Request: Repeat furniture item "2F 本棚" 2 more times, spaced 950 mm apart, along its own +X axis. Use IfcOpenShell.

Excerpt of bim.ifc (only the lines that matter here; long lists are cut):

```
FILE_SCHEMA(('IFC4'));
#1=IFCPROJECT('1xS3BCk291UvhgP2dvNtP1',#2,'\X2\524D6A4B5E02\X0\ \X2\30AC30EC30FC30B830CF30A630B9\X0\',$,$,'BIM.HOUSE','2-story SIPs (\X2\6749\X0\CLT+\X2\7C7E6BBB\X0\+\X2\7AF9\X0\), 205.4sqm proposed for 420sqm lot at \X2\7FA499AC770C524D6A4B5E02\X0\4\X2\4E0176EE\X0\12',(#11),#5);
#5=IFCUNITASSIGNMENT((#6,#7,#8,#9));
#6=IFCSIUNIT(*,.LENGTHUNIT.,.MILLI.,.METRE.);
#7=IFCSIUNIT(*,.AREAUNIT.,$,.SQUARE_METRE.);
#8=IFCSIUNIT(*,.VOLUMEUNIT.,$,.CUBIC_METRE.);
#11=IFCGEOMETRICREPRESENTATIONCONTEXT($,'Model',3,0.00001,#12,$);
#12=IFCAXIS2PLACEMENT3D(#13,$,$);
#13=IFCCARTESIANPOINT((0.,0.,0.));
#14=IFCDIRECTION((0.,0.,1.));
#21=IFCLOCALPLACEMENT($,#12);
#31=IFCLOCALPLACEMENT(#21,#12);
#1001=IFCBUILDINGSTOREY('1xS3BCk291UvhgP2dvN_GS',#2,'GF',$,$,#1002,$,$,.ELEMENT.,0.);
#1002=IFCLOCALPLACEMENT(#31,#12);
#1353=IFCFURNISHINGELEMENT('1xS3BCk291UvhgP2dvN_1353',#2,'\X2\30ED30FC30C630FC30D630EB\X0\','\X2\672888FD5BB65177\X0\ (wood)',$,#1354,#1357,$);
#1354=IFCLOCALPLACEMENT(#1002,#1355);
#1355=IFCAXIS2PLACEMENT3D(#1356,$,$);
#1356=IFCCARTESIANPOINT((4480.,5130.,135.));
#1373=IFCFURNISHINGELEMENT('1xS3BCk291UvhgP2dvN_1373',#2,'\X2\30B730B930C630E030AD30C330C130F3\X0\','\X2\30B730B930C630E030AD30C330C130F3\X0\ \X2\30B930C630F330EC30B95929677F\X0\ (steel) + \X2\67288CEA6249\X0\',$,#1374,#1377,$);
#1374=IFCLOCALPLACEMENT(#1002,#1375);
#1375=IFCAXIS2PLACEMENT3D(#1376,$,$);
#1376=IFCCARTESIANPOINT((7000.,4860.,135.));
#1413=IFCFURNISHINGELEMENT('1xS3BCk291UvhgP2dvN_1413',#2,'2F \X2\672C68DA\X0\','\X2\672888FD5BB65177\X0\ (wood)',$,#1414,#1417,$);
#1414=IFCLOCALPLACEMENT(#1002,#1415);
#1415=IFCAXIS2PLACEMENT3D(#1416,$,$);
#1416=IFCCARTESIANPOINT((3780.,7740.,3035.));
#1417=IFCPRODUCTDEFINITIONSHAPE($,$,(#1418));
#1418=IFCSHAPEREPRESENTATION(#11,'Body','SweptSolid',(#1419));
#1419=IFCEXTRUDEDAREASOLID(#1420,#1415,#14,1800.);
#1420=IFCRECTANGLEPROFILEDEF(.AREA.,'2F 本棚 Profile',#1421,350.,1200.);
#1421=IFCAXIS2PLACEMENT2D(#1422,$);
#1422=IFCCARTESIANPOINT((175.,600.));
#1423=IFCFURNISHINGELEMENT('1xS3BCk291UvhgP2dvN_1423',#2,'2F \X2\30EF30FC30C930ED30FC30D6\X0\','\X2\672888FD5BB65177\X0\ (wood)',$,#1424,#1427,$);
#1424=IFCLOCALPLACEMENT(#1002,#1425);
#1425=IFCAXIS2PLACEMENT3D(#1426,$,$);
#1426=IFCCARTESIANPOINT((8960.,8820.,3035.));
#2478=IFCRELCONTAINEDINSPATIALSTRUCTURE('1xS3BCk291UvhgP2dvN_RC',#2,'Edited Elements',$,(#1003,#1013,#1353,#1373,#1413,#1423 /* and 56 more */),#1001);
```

```python
import ifcopenshell
import ifcopenshell.api.geometry
import ifcopenshell.api.root
import ifcopenshell.util.element
import ifcopenshell.util.placement
import ifcopenshell.util.unit

model = ifcopenshell.open("bim.ifc")
unit_scale = ifcopenshell.util.unit.calculate_unit_scale(model)


def reuse_history(source, copy):
    """copy_class also copies each property set's owner history, people and application; keep the originals."""
    for rel in copy.IsDefinedBy:
        if rel.is_a("IfcRelDefinesByProperties") and (history := rel.RelatingPropertyDefinition.OwnerHistory):
            rel.RelatingPropertyDefinition.OwnerHistory = source.OwnerHistory
            ifcopenshell.util.element.remove_deep2(model, history)


source = model.by_id(1413)
base = ifcopenshell.util.placement.get_local_placement(source.ObjectPlacement)
step = base[:3, 0] * 0.95 / unit_scale

for i in range(1, 3):
    copy = ifcopenshell.api.root.copy_class(model, product=source)
    copy.Representation = ifcopenshell.util.element.copy_deep(
        model, source.Representation, exclude=["IfcGeometricRepresentationContext", "IfcRepresentationMap"]
    )
    reuse_history(source, copy)
    matrix = base.copy()
    matrix[:3, 3] += i * step
    print("added at", matrix[:3, 3].round(3) + 0.0)
    ifcopenshell.api.geometry.edit_object_placement(model, product=copy, matrix=matrix, is_si=False)

model.write("bim_edited.ifc")
```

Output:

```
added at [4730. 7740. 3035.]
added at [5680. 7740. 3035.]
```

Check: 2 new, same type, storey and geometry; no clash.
